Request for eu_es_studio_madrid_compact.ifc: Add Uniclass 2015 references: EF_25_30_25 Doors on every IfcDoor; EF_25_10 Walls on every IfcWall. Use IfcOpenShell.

First a look at what the model holds.

```python
import ifcopenshell

model = ifcopenshell.open("eu_es_studio_madrid_compact.ifc")
print(model.schema)
print("classifications:", [c.Name for c in model.by_type("IfcClassification")])
for ifc_class in ("IfcDoor", "IfcRoof", "IfcStair", "IfcWall", "IfcWindow"):
    print(ifc_class, len(model.by_type(ifc_class)))
```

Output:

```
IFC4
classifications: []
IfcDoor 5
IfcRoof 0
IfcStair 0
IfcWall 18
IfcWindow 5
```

```python
import ifcopenshell
import ifcopenshell.api.classification

model = ifcopenshell.open("eu_es_studio_madrid_compact.ifc")

system = ifcopenshell.api.classification.add_classification(model, classification="Uniclass 2015")

codes = {
    "IfcDoor": ("EF_25_30_25", "Doors"),
    "IfcWall": ("EF_25_10", "Walls"),
}
for ifc_class, (code, name) in codes.items():
    products = model.by_type(ifc_class)
    ifcopenshell.api.classification.add_reference(
        model, products=products, classification=system, identification=code, name=name
    )
    print(code, len(products))

model.write("eu_es_studio_madrid_compact_rev.ifc")
```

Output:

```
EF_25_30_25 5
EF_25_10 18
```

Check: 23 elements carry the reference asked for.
